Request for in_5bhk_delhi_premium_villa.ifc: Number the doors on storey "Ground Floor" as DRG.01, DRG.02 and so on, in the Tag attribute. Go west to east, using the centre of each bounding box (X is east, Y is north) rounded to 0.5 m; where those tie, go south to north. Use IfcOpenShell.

First a look at what the model holds.

```python
import ifcopenshell
import ifcopenshell.util.element
import ifcopenshell.util.placement

model = ifcopenshell.open("in_5bhk_delhi_premium_villa.ifc")
print(model.schema)
storey = next(s for s in model.by_type("IfcBuildingStorey") if s.Name == "Ground Floor")
doors = [e for e in ifcopenshell.util.element.get_decomposition(storey) if e.is_a("IfcDoor")]
for e in sorted(doors, key=lambda e: e.id()):
    origin = ifcopenshell.util.placement.get_local_placement(e.ObjectPlacement)[:3, 3]
    print(e.id(), e.Tag, e.Name, origin.round(2) + 0.0, sep=" | ")
```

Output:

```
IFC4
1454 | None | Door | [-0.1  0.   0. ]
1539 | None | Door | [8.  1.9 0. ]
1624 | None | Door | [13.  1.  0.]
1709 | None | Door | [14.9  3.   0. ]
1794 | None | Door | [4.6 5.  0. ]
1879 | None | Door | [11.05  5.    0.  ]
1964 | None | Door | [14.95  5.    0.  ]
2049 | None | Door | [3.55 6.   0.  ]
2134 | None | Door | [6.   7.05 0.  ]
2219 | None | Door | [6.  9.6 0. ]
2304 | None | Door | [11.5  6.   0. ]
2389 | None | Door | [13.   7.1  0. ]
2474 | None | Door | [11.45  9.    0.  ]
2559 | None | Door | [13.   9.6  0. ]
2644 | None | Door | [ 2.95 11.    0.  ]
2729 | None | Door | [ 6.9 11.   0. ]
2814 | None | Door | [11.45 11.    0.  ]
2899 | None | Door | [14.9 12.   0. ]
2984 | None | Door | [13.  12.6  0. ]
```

```python
import ifcopenshell
import ifcopenshell.geom
import ifcopenshell.util.element
import ifcopenshell.util.shape

model = ifcopenshell.open("in_5bhk_delhi_premium_villa.ifc")
settings = ifcopenshell.geom.settings()
settings.set("use-world-coords", True)


def centre(element):
    shape = ifcopenshell.geom.create_shape(settings, element)
    return ifcopenshell.util.shape.get_bbox_centroid(shape.geometry)


storey = next(s for s in model.by_type("IfcBuildingStorey") if s.Name == "Ground Floor")
doors = [e for e in ifcopenshell.util.element.get_decomposition(storey) if e.is_a("IfcDoor")]

# Insertion points can sit at a corner or the storey origin, so sort by the geometry (in metres).
centres = {e: centre(e) for e in doors}
doors.sort(key=lambda e: (round(centres[e][0] / 0.5), centres[e][1]))

for i, e in enumerate(doors, start=1):
    number = f"DRG.{i:02d}"
    e.Tag = number
    print(e.id(), number)

model.write("in_5bhk_delhi_premium_villa_rev.ifc")
```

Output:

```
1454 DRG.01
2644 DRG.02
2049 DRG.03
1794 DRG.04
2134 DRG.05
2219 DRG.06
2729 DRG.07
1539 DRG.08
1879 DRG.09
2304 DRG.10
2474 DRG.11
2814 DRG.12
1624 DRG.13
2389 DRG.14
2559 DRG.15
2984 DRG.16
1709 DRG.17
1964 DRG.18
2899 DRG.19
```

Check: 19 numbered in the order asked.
